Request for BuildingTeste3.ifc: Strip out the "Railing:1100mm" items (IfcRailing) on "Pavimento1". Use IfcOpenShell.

First a look at what the model holds.

```python
import ifcopenshell
import ifcopenshell.util.element

model = ifcopenshell.open("BuildingTeste3.ifc")
print(model.schema)
storey = next(s for s in model.by_type("IfcBuildingStorey") if s.Name == "Pavimento1")
railings = [e for e in ifcopenshell.util.element.get_decomposition(storey) if e.is_a("IfcRailing")]
seen = {}
for e in railings:
    element_type = ifcopenshell.util.element.get_type(e)
    name = element_type.Name if element_type not in (None, e) else None
    seen[name] = seen.get(name, 0) + 1
for name, count in sorted(seen.items(), key=str):
    print(count, "x", name)
```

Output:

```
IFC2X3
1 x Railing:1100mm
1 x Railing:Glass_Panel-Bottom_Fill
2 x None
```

```python
import ifcopenshell
import ifcopenshell.api.root
import ifcopenshell.util.element

model = ifcopenshell.open("BuildingTeste3.ifc")

storey = next(s for s in model.by_type("IfcBuildingStorey") if s.Name == "Pavimento1")
railings = [e for e in ifcopenshell.util.element.get_decomposition(storey) if e.is_a("IfcRailing")]
targets = [e for e in railings if (t := ifcopenshell.util.element.get_type(e)) not in (None, e) and t.Name == "Railing:1100mm"]

for e in targets:
    ifcopenshell.api.root.remove_product(model, product=e)
print(len(targets), "removed")

model.write("BuildingTeste3-out.ifc")
```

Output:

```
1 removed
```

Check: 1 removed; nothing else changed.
